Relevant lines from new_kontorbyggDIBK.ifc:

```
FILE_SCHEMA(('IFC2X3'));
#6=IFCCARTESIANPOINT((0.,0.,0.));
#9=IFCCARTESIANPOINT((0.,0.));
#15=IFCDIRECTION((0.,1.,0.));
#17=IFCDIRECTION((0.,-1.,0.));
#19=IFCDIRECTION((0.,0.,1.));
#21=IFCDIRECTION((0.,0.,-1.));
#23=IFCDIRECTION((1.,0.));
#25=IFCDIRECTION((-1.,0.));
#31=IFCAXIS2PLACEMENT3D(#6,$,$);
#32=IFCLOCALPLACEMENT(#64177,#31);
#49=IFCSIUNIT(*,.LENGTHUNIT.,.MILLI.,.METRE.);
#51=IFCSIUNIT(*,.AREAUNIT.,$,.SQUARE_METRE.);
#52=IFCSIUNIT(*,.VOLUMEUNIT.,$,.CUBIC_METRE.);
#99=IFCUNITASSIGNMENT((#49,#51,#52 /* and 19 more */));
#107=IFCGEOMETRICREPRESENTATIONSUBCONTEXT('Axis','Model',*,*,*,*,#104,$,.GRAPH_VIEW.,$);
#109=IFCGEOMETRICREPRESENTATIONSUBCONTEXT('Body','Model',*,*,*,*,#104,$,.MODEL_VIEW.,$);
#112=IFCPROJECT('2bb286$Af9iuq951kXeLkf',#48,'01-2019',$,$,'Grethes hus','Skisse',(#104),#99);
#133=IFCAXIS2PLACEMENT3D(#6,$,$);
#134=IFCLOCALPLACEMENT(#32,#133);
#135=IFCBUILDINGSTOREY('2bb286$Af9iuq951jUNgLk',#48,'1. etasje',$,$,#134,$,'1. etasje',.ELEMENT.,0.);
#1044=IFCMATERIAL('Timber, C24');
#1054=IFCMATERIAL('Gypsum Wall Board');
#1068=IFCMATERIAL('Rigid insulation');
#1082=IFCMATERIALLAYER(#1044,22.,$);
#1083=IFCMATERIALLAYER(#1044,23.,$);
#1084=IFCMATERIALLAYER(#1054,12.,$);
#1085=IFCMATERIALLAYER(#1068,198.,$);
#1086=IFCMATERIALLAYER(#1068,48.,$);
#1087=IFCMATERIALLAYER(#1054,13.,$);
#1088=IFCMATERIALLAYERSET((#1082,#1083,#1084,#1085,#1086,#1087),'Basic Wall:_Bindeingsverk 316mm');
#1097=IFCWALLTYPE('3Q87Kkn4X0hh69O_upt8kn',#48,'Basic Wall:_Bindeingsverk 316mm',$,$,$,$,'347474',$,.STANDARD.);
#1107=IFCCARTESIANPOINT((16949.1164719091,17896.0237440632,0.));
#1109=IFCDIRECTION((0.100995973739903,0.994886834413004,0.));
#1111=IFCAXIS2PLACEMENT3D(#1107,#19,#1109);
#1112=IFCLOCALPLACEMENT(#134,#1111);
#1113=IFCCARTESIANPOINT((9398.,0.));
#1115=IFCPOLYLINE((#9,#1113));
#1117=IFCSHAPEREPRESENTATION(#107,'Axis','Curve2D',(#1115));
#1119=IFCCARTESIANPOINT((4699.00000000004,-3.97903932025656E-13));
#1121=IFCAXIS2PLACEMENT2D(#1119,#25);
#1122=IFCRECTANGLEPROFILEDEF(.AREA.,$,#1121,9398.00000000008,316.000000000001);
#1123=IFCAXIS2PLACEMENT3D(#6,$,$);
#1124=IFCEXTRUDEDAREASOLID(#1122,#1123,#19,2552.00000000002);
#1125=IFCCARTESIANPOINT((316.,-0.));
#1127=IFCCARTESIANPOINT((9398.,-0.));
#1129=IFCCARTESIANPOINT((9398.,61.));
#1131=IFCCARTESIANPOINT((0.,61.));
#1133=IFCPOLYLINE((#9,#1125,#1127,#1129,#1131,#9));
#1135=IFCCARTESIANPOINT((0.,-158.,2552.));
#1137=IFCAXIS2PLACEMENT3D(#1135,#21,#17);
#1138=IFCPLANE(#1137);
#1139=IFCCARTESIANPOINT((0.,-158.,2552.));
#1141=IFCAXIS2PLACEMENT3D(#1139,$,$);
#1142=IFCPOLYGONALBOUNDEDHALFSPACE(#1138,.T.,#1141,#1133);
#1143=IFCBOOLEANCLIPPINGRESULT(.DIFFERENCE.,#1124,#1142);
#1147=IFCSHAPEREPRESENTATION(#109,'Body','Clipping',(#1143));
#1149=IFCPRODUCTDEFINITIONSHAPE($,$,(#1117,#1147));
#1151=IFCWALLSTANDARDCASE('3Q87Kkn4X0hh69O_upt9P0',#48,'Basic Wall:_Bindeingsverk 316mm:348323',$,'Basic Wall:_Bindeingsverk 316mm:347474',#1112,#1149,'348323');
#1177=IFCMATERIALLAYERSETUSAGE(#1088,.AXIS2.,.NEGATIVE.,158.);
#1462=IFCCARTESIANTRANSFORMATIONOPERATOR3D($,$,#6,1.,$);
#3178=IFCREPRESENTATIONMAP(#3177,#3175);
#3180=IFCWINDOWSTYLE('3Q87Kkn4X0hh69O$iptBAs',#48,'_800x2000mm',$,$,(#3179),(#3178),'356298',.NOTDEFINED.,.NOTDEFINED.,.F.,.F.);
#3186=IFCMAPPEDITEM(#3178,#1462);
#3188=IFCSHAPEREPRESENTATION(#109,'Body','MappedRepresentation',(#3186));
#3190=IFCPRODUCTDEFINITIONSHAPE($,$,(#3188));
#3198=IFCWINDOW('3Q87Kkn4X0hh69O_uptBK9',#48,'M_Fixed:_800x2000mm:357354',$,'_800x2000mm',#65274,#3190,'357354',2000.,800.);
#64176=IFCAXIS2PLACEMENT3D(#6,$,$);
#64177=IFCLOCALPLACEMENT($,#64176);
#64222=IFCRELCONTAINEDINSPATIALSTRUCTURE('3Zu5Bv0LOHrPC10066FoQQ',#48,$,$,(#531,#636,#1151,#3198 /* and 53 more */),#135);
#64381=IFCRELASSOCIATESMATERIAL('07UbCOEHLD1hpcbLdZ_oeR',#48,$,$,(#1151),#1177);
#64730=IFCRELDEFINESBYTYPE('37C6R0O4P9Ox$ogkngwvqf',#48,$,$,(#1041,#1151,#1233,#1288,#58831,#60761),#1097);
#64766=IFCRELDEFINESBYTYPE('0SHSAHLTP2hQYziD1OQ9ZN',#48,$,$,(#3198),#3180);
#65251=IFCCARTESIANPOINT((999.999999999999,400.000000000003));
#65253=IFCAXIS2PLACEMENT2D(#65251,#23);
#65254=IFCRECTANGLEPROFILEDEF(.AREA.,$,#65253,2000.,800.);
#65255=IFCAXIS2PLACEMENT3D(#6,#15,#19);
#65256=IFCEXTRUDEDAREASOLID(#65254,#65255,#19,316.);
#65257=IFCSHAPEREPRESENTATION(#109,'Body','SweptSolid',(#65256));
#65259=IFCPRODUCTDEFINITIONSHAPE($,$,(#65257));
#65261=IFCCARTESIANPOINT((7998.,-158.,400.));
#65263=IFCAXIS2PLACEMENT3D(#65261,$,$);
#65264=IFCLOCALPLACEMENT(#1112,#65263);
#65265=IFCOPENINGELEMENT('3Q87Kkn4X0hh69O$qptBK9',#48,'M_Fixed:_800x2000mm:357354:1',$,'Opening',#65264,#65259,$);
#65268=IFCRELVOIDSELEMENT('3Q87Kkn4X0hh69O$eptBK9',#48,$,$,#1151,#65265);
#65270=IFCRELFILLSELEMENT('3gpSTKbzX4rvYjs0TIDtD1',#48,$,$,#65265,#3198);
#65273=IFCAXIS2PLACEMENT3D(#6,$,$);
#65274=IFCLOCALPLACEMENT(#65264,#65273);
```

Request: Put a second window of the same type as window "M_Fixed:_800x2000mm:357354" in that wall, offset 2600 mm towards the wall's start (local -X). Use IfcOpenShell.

```python
import ifcopenshell
import ifcopenshell.api.feature
import ifcopenshell.api.geometry
import ifcopenshell.api.root
import ifcopenshell.geom
import ifcopenshell.util.element
import ifcopenshell.util.placement
import ifcopenshell.util.shape
import ifcopenshell.util.unit

model = ifcopenshell.open("new_kontorbyggDIBK.ifc")
unit_scale = ifcopenshell.util.unit.calculate_unit_scale(model)
settings = ifcopenshell.geom.settings()


def volume(element):
    """Net volume in cubic metres, openings subtracted."""
    shape = ifcopenshell.geom.create_shape(settings, element)
    return ifcopenshell.util.shape.get_volume(shape.geometry)


def reuse_history(source, copy):
    """copy_class also copies each property set's owner history, people and application; keep the originals."""
    for rel in copy.IsDefinedBy:
        if rel.is_a("IfcRelDefinesByProperties") and (history := rel.RelatingPropertyDefinition.OwnerHistory):
            rel.RelatingPropertyDefinition.OwnerHistory = source.OwnerHistory
            ifcopenshell.util.element.remove_deep2(model, history)


window = model.by_id(3198)
opening = window.FillsVoids[0].RelatingOpeningElement
wall = opening.VoidsElements[0].RelatingBuildingElement
before = volume(wall)
shift = ifcopenshell.util.placement.get_local_placement(wall.ObjectPlacement)[:3, 0] * -2.6 / unit_scale

# copy_class copies the void relationship, type, container and properties, but no geometry.
new_opening = ifcopenshell.api.root.copy_class(model, product=opening)
new_opening.Representation = ifcopenshell.util.element.copy_deep(
    model, opening.Representation, exclude=["IfcGeometricRepresentationContext", "IfcRepresentationMap"]
)
new_opening.Name = "M_Fixed:_800x2000mm"
new_window = ifcopenshell.api.root.copy_class(model, product=window)
new_window.Representation = ifcopenshell.util.element.copy_deep(
    model, window.Representation, exclude=["IfcGeometricRepresentationContext", "IfcRepresentationMap"]
)
new_window.Name = "M_Fixed:_800x2000mm"
new_window.Tag = None
reuse_history(window, new_window)
fills = ifcopenshell.api.feature.add_filling(model, opening=new_opening, element=new_window)
fills.OwnerHistory = new_window.OwnerHistory  # required in IFC2X3

for old, new in ((opening, new_opening), (window, new_window)):
    matrix = ifcopenshell.util.placement.get_local_placement(old.ObjectPlacement)
    matrix[:3, 3] += shift
    ifcopenshell.api.geometry.edit_object_placement(model, product=new, matrix=matrix, is_si=False)

after = volume(wall)

print(f"wall volume {before:.3f} -> {after:.3f} m3")

model.write("new_kontorbyggDIBK_v2.ifc")
```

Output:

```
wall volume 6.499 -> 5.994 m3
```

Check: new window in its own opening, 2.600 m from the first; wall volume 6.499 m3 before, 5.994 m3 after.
